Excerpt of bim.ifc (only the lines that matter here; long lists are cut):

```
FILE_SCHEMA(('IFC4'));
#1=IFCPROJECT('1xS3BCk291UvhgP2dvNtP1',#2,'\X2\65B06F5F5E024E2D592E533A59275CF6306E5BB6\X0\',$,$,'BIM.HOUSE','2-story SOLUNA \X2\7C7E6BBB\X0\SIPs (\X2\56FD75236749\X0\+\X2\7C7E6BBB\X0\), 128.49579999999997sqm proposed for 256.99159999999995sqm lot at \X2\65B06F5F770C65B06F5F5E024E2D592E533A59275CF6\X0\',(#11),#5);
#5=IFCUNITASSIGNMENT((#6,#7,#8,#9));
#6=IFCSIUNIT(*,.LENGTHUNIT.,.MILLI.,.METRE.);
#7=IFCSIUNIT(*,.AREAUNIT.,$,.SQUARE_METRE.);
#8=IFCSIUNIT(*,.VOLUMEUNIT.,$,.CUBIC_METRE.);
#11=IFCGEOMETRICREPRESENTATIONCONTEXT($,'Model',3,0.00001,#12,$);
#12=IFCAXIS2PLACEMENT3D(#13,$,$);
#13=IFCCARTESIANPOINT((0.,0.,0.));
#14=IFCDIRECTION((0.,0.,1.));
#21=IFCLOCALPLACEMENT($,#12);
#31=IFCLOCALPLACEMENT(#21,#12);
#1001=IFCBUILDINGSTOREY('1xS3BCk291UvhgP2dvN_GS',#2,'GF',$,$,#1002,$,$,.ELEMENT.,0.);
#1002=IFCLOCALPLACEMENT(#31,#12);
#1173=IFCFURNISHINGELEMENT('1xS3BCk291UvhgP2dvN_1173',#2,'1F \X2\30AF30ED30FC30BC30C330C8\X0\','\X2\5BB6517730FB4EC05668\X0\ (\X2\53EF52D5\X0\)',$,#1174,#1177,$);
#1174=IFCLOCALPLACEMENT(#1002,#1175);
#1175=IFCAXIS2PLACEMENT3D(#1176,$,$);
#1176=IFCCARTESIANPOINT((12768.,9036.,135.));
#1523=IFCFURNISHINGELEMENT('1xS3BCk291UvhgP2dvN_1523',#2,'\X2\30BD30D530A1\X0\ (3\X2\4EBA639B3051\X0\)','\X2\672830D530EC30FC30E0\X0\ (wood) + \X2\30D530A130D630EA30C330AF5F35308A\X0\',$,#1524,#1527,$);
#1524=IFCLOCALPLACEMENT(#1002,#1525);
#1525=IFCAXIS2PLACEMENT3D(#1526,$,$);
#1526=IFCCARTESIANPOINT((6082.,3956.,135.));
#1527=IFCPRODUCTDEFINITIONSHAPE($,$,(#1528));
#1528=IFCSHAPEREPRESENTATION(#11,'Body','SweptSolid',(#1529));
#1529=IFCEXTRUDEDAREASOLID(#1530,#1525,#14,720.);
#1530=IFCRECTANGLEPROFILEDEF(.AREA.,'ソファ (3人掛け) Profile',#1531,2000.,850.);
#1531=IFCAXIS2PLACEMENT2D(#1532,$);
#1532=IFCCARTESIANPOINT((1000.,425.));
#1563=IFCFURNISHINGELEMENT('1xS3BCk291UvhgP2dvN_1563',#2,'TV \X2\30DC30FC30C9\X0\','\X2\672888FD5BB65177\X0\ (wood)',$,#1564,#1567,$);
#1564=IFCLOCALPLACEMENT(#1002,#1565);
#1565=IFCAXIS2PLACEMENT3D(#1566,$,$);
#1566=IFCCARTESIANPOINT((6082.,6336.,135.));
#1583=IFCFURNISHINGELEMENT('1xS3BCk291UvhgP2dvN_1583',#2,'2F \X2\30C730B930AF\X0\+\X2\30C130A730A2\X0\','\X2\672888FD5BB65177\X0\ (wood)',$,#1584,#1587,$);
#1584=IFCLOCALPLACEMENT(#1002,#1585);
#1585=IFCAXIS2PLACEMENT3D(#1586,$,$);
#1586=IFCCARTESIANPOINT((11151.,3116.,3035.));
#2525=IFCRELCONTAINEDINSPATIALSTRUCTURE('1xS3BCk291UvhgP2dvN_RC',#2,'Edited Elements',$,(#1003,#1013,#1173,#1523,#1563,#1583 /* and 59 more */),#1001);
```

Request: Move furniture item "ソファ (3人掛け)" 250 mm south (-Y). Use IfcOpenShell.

```python
import ifcopenshell
import ifcopenshell.api.geometry
import ifcopenshell.util.placement
import ifcopenshell.util.unit

model = ifcopenshell.open("bim.ifc")
unit_scale = ifcopenshell.util.unit.calculate_unit_scale(model)

item = model.by_id(1523)
matrix = ifcopenshell.util.placement.get_local_placement(item.ObjectPlacement)
matrix[1, 3] -= 0.25 / unit_scale
ifcopenshell.api.geometry.edit_object_placement(model, product=item, matrix=matrix, is_si=False)

print(ifcopenshell.util.placement.get_local_placement(item.ObjectPlacement).round(3) + 0.0)

model.write("bim-out.ifc")
```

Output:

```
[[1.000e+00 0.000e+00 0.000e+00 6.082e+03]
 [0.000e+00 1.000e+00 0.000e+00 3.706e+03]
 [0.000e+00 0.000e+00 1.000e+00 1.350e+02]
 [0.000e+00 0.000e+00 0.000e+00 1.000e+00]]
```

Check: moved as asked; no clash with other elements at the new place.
